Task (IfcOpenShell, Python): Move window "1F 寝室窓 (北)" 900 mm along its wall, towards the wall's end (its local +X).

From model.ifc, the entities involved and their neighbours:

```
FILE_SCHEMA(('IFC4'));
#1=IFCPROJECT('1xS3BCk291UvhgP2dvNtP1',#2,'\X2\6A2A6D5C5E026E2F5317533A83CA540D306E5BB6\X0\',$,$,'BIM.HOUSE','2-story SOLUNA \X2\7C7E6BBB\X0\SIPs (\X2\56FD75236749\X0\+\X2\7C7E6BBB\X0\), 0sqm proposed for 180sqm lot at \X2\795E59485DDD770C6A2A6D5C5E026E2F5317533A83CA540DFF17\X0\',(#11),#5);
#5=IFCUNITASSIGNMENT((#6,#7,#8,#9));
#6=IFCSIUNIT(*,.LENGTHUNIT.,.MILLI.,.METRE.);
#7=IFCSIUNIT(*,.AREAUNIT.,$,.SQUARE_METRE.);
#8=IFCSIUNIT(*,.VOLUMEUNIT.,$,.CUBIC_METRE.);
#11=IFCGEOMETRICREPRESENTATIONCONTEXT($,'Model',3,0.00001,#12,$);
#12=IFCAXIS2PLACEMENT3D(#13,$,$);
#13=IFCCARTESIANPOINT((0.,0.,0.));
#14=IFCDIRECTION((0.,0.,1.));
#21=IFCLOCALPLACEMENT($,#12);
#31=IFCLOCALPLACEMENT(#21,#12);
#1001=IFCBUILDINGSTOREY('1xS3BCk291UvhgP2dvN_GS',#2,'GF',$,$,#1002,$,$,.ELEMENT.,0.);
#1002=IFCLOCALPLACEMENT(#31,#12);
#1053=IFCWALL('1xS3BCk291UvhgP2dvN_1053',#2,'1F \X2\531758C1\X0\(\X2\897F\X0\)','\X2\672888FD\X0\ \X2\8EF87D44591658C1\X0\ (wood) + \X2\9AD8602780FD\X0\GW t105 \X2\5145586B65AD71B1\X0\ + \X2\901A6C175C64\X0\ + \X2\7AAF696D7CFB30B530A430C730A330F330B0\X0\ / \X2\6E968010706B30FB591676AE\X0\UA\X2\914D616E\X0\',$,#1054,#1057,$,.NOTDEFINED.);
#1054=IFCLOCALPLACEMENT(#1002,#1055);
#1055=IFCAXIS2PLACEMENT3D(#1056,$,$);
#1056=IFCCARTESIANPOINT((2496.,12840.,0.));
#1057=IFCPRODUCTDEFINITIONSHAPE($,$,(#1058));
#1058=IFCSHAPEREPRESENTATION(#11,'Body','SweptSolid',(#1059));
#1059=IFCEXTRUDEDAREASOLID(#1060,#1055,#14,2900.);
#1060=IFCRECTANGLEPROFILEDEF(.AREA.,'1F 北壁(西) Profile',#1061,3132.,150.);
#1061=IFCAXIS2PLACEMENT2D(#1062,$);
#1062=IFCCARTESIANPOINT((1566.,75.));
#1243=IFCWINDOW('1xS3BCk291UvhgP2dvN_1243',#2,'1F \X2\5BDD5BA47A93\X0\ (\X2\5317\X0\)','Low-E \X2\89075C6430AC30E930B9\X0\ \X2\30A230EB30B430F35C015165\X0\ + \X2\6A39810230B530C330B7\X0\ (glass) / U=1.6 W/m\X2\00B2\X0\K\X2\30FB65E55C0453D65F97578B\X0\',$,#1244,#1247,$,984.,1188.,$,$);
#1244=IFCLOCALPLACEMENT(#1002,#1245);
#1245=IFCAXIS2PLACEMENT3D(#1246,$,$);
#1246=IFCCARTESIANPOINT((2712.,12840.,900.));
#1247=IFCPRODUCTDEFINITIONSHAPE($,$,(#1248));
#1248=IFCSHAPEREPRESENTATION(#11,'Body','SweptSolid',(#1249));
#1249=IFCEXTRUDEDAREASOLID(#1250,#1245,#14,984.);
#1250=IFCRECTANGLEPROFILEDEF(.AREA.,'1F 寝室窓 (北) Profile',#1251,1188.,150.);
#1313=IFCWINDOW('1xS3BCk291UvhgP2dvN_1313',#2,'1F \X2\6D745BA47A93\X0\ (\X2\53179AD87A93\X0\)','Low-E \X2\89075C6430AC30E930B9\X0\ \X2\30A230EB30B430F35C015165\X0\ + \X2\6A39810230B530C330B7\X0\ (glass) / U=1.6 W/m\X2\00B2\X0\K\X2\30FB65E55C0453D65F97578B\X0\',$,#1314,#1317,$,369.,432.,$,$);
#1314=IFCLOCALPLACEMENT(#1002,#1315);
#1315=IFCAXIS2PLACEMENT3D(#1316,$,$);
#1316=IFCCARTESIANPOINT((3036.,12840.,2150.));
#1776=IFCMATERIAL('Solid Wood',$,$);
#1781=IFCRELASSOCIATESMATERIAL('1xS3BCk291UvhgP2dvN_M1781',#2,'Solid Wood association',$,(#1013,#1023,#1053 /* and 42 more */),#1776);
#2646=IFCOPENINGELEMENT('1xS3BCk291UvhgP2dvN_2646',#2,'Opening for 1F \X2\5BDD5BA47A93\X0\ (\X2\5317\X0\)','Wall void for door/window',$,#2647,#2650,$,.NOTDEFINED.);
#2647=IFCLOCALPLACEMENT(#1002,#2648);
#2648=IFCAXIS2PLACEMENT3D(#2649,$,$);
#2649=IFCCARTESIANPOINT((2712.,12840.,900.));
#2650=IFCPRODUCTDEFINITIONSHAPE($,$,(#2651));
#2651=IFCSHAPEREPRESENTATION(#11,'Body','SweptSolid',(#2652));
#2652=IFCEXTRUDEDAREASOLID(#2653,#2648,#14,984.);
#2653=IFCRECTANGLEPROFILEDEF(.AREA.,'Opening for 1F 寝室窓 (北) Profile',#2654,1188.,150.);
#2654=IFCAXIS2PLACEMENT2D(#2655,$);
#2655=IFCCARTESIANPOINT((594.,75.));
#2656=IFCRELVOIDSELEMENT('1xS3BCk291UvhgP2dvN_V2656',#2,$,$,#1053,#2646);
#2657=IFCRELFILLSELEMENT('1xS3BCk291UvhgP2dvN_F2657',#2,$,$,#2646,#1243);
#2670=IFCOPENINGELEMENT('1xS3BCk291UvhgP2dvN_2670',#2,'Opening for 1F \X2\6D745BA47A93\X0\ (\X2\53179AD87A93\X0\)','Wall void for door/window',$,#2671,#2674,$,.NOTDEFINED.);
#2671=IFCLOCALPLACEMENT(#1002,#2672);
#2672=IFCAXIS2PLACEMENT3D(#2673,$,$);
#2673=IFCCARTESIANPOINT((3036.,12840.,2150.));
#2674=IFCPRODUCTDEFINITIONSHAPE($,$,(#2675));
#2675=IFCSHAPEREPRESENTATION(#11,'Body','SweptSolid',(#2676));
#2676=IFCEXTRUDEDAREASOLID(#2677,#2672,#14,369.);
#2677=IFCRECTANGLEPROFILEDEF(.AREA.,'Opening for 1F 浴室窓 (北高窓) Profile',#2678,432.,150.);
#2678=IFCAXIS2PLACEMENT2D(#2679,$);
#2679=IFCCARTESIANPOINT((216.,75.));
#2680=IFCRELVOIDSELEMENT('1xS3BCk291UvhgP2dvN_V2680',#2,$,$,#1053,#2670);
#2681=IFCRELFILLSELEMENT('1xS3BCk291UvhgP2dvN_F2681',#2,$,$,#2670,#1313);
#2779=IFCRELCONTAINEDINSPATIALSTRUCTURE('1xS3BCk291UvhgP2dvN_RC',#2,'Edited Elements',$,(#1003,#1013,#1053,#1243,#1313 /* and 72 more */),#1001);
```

```python
import ifcopenshell
import ifcopenshell.api.geometry
import ifcopenshell.util.placement

model = ifcopenshell.open("model.ifc")

window = model.by_id(1243)
opening = window.FillsVoids[0].RelatingOpeningElement
wall = opening.VoidsElements[0].RelatingBuildingElement

wall_matrix = ifcopenshell.util.placement.get_local_placement(wall.ObjectPlacement)
shift = wall_matrix[:3, 0] * 900.0
before = ifcopenshell.util.placement.get_local_placement(window.ObjectPlacement)[:3, 3].copy()

# The window is not placed relative to its opening, so move both.
for product in (opening, window):
    matrix = ifcopenshell.util.placement.get_local_placement(product.ObjectPlacement)
    matrix[:3, 3] += shift
    ifcopenshell.api.geometry.edit_object_placement(model, product=product, matrix=matrix, is_si=False)

after = ifcopenshell.util.placement.get_local_placement(window.ObjectPlacement)[:3, 3]
print("window moved by", (after - before).round(3) + 0.0)

model.write("model_edited.ifc")
```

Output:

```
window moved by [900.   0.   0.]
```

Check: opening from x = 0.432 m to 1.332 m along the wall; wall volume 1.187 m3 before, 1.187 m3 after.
